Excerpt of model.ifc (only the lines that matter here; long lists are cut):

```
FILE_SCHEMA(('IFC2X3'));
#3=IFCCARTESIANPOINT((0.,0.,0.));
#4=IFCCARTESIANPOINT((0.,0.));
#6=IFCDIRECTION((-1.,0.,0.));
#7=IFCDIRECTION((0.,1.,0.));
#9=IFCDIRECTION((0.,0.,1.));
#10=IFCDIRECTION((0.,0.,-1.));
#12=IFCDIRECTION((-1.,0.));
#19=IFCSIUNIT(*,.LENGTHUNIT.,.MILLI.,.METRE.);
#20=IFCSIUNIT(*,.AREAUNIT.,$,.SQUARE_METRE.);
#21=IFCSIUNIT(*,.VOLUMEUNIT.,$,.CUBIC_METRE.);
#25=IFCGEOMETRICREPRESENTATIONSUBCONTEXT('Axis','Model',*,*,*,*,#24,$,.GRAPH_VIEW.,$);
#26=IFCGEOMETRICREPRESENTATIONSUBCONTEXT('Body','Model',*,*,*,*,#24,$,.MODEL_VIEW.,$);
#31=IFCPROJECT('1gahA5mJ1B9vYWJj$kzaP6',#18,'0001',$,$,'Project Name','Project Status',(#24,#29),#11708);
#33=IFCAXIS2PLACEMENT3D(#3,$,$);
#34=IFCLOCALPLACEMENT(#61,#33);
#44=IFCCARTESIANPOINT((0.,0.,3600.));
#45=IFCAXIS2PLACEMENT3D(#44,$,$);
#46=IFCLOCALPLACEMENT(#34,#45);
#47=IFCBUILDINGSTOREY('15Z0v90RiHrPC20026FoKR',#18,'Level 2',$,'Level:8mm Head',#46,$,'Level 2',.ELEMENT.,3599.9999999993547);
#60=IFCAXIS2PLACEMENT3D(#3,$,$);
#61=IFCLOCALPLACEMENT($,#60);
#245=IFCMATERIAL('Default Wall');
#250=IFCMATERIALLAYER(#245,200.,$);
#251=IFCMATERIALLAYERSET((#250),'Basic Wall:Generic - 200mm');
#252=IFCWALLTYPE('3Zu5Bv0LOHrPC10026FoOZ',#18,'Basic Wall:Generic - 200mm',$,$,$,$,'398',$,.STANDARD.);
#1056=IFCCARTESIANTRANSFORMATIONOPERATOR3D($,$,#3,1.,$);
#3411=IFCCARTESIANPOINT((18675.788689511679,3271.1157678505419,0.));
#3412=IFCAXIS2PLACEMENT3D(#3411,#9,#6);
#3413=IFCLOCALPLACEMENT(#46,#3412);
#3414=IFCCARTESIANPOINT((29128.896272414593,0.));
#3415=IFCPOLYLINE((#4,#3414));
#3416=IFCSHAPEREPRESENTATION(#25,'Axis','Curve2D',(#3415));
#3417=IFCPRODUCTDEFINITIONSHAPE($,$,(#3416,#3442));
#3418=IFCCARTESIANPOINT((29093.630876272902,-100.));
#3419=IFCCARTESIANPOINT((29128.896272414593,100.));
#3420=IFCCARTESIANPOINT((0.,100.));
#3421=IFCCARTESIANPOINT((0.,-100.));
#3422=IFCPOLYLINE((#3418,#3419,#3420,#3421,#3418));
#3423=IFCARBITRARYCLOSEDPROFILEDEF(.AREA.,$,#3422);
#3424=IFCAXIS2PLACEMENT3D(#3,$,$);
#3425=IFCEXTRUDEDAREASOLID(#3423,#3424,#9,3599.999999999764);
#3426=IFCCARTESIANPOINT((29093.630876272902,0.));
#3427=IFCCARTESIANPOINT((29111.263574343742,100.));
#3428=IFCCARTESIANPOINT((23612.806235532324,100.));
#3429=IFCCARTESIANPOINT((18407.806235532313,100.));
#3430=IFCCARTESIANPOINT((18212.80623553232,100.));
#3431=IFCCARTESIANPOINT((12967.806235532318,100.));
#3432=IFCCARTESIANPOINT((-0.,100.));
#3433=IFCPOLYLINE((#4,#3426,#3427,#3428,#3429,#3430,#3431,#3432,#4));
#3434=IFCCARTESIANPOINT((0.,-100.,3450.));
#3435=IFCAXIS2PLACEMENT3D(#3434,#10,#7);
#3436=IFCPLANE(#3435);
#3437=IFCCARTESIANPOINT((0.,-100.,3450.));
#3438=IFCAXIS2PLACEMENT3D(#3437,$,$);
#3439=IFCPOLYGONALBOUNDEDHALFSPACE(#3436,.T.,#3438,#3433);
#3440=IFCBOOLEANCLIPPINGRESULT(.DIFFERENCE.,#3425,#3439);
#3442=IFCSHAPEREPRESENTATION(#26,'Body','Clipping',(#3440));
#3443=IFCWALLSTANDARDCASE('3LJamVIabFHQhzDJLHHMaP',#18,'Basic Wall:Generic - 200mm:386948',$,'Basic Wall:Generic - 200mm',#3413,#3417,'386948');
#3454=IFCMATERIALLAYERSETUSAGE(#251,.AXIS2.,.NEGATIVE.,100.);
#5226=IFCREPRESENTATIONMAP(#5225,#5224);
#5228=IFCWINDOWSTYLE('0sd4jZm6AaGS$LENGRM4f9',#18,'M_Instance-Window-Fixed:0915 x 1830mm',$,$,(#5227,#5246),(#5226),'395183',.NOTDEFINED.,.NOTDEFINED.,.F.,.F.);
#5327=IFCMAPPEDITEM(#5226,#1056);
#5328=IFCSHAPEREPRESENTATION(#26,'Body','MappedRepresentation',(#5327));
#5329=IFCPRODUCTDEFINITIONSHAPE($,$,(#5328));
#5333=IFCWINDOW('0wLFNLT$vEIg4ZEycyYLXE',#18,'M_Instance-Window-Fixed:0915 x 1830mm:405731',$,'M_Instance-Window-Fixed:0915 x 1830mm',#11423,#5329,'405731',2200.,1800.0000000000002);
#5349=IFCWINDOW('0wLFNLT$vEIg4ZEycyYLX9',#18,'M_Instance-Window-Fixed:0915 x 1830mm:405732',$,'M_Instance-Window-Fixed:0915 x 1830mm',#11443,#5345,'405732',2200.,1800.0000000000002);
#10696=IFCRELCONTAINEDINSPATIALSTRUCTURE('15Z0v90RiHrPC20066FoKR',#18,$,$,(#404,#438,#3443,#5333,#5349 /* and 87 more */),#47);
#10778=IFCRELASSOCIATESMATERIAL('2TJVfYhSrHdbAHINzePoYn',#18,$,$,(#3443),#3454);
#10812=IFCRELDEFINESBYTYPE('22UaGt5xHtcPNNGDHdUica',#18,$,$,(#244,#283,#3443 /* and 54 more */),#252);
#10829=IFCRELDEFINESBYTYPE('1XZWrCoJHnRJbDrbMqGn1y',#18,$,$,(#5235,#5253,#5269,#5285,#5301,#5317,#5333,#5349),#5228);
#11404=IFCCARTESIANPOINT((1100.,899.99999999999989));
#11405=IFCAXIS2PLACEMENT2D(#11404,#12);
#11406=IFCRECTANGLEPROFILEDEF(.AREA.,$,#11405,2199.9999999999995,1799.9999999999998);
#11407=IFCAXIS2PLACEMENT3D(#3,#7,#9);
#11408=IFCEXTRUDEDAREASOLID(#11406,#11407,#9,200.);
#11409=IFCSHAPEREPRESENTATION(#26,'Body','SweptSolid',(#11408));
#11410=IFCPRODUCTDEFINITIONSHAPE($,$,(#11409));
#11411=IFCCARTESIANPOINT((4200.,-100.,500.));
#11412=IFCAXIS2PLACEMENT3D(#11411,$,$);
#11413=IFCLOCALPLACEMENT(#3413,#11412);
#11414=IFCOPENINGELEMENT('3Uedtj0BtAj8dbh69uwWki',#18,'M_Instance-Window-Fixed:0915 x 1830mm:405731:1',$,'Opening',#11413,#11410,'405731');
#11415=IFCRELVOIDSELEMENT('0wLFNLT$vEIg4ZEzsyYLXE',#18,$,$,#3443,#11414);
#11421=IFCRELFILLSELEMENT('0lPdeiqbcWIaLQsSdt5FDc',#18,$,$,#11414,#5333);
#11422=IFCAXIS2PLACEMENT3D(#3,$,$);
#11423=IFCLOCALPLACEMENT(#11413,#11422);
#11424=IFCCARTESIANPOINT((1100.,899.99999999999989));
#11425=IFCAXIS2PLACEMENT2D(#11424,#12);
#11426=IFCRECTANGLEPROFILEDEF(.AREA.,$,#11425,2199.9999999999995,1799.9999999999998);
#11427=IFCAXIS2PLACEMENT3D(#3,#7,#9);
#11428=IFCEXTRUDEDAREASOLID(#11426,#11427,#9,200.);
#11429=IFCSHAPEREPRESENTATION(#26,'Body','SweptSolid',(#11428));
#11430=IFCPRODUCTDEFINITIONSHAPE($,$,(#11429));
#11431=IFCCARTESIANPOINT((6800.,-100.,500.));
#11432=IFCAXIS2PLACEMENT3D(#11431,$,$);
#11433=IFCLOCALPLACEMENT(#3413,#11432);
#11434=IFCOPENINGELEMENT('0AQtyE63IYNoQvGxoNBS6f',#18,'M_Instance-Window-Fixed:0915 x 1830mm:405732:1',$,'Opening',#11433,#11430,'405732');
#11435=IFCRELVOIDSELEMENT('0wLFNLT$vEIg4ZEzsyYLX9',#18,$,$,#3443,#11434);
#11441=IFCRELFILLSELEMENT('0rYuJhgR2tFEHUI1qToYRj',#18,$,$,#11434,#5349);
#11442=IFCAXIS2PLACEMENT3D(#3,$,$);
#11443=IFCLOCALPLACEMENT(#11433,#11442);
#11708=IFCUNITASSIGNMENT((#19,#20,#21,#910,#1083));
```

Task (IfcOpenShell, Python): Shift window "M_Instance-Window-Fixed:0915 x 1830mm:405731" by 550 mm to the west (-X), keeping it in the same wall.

```python
import ifcopenshell
import ifcopenshell.api.geometry
import ifcopenshell.util.placement
import ifcopenshell.util.unit

model = ifcopenshell.open("model.ifc")
unit_scale = ifcopenshell.util.unit.calculate_unit_scale(model)

window = model.by_guid("0wLFNLT$vEIg4ZEycyYLXE")
opening = window.FillsVoids[0].RelatingOpeningElement
wall = opening.VoidsElements[0].RelatingBuildingElement

wall_matrix = ifcopenshell.util.placement.get_local_placement(wall.ObjectPlacement)
shift = wall_matrix[:3, 0] * 0.55 / unit_scale
before = ifcopenshell.util.placement.get_local_placement(window.ObjectPlacement)[:3, 3].copy()

# The window is placed relative to its opening, so it follows when the opening moves.
matrix = ifcopenshell.util.placement.get_local_placement(opening.ObjectPlacement)
matrix[:3, 3] += shift
ifcopenshell.api.geometry.edit_object_placement(
    model, product=opening, matrix=matrix, is_si=False, should_transform_children=True
)

after = ifcopenshell.util.placement.get_local_placement(window.ObjectPlacement)[:3, 3]
print("window moved by", (after - before).round(3) + 0.0)

model.write("model_updated.ifc")
```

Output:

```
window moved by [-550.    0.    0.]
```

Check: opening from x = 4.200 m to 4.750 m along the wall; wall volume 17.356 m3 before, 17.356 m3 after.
